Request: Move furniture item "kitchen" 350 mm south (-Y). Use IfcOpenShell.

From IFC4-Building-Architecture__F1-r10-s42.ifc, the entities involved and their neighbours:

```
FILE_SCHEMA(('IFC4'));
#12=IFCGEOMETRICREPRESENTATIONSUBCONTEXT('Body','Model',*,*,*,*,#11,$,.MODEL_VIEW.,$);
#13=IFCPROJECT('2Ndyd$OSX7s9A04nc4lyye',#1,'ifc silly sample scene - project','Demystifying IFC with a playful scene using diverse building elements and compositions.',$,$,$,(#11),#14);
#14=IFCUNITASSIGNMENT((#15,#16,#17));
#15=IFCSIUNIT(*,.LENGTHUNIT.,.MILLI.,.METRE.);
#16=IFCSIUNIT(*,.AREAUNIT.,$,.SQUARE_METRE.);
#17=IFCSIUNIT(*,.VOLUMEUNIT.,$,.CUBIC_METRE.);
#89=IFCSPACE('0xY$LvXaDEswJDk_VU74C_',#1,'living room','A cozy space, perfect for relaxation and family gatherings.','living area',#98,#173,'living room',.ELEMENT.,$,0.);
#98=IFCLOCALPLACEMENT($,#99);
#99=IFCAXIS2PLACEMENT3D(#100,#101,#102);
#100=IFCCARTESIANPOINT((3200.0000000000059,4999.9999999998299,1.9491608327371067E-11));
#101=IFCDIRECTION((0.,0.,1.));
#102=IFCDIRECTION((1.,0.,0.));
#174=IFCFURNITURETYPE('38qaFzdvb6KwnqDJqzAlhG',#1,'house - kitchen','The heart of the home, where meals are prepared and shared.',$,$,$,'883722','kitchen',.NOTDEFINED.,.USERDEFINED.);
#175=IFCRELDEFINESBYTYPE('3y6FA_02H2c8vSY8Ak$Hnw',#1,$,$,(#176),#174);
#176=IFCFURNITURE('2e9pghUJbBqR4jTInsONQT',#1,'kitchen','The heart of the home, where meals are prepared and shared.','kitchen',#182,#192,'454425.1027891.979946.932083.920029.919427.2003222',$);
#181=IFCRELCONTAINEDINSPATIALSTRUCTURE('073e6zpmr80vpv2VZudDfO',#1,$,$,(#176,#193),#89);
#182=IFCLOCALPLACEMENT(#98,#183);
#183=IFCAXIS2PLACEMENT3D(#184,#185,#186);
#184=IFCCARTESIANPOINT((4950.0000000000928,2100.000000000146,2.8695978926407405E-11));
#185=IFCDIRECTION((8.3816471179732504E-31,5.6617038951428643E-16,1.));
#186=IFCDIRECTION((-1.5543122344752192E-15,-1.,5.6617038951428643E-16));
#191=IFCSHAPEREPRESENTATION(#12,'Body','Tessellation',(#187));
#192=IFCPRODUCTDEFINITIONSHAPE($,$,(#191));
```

```python
import ifcopenshell
import ifcopenshell.api.geometry
import ifcopenshell.util.placement
import ifcopenshell.util.unit

model = ifcopenshell.open("IFC4-Building-Architecture__F1-r10-s42.ifc")
unit_scale = ifcopenshell.util.unit.calculate_unit_scale(model)

item = model.by_id(176)
matrix = ifcopenshell.util.placement.get_local_placement(item.ObjectPlacement)
matrix[1, 3] -= 0.35 / unit_scale
ifcopenshell.api.geometry.edit_object_placement(model, product=item, matrix=matrix, is_si=False)

print(ifcopenshell.util.placement.get_local_placement(item.ObjectPlacement).round(3) + 0.0)

model.write("IFC4-Building-Architecture__F1-r10-s42-out.ifc")
```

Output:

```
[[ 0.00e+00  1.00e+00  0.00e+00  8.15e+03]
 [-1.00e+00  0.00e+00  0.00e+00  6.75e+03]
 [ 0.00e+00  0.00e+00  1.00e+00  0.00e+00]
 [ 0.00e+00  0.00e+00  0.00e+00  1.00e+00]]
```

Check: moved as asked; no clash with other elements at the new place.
